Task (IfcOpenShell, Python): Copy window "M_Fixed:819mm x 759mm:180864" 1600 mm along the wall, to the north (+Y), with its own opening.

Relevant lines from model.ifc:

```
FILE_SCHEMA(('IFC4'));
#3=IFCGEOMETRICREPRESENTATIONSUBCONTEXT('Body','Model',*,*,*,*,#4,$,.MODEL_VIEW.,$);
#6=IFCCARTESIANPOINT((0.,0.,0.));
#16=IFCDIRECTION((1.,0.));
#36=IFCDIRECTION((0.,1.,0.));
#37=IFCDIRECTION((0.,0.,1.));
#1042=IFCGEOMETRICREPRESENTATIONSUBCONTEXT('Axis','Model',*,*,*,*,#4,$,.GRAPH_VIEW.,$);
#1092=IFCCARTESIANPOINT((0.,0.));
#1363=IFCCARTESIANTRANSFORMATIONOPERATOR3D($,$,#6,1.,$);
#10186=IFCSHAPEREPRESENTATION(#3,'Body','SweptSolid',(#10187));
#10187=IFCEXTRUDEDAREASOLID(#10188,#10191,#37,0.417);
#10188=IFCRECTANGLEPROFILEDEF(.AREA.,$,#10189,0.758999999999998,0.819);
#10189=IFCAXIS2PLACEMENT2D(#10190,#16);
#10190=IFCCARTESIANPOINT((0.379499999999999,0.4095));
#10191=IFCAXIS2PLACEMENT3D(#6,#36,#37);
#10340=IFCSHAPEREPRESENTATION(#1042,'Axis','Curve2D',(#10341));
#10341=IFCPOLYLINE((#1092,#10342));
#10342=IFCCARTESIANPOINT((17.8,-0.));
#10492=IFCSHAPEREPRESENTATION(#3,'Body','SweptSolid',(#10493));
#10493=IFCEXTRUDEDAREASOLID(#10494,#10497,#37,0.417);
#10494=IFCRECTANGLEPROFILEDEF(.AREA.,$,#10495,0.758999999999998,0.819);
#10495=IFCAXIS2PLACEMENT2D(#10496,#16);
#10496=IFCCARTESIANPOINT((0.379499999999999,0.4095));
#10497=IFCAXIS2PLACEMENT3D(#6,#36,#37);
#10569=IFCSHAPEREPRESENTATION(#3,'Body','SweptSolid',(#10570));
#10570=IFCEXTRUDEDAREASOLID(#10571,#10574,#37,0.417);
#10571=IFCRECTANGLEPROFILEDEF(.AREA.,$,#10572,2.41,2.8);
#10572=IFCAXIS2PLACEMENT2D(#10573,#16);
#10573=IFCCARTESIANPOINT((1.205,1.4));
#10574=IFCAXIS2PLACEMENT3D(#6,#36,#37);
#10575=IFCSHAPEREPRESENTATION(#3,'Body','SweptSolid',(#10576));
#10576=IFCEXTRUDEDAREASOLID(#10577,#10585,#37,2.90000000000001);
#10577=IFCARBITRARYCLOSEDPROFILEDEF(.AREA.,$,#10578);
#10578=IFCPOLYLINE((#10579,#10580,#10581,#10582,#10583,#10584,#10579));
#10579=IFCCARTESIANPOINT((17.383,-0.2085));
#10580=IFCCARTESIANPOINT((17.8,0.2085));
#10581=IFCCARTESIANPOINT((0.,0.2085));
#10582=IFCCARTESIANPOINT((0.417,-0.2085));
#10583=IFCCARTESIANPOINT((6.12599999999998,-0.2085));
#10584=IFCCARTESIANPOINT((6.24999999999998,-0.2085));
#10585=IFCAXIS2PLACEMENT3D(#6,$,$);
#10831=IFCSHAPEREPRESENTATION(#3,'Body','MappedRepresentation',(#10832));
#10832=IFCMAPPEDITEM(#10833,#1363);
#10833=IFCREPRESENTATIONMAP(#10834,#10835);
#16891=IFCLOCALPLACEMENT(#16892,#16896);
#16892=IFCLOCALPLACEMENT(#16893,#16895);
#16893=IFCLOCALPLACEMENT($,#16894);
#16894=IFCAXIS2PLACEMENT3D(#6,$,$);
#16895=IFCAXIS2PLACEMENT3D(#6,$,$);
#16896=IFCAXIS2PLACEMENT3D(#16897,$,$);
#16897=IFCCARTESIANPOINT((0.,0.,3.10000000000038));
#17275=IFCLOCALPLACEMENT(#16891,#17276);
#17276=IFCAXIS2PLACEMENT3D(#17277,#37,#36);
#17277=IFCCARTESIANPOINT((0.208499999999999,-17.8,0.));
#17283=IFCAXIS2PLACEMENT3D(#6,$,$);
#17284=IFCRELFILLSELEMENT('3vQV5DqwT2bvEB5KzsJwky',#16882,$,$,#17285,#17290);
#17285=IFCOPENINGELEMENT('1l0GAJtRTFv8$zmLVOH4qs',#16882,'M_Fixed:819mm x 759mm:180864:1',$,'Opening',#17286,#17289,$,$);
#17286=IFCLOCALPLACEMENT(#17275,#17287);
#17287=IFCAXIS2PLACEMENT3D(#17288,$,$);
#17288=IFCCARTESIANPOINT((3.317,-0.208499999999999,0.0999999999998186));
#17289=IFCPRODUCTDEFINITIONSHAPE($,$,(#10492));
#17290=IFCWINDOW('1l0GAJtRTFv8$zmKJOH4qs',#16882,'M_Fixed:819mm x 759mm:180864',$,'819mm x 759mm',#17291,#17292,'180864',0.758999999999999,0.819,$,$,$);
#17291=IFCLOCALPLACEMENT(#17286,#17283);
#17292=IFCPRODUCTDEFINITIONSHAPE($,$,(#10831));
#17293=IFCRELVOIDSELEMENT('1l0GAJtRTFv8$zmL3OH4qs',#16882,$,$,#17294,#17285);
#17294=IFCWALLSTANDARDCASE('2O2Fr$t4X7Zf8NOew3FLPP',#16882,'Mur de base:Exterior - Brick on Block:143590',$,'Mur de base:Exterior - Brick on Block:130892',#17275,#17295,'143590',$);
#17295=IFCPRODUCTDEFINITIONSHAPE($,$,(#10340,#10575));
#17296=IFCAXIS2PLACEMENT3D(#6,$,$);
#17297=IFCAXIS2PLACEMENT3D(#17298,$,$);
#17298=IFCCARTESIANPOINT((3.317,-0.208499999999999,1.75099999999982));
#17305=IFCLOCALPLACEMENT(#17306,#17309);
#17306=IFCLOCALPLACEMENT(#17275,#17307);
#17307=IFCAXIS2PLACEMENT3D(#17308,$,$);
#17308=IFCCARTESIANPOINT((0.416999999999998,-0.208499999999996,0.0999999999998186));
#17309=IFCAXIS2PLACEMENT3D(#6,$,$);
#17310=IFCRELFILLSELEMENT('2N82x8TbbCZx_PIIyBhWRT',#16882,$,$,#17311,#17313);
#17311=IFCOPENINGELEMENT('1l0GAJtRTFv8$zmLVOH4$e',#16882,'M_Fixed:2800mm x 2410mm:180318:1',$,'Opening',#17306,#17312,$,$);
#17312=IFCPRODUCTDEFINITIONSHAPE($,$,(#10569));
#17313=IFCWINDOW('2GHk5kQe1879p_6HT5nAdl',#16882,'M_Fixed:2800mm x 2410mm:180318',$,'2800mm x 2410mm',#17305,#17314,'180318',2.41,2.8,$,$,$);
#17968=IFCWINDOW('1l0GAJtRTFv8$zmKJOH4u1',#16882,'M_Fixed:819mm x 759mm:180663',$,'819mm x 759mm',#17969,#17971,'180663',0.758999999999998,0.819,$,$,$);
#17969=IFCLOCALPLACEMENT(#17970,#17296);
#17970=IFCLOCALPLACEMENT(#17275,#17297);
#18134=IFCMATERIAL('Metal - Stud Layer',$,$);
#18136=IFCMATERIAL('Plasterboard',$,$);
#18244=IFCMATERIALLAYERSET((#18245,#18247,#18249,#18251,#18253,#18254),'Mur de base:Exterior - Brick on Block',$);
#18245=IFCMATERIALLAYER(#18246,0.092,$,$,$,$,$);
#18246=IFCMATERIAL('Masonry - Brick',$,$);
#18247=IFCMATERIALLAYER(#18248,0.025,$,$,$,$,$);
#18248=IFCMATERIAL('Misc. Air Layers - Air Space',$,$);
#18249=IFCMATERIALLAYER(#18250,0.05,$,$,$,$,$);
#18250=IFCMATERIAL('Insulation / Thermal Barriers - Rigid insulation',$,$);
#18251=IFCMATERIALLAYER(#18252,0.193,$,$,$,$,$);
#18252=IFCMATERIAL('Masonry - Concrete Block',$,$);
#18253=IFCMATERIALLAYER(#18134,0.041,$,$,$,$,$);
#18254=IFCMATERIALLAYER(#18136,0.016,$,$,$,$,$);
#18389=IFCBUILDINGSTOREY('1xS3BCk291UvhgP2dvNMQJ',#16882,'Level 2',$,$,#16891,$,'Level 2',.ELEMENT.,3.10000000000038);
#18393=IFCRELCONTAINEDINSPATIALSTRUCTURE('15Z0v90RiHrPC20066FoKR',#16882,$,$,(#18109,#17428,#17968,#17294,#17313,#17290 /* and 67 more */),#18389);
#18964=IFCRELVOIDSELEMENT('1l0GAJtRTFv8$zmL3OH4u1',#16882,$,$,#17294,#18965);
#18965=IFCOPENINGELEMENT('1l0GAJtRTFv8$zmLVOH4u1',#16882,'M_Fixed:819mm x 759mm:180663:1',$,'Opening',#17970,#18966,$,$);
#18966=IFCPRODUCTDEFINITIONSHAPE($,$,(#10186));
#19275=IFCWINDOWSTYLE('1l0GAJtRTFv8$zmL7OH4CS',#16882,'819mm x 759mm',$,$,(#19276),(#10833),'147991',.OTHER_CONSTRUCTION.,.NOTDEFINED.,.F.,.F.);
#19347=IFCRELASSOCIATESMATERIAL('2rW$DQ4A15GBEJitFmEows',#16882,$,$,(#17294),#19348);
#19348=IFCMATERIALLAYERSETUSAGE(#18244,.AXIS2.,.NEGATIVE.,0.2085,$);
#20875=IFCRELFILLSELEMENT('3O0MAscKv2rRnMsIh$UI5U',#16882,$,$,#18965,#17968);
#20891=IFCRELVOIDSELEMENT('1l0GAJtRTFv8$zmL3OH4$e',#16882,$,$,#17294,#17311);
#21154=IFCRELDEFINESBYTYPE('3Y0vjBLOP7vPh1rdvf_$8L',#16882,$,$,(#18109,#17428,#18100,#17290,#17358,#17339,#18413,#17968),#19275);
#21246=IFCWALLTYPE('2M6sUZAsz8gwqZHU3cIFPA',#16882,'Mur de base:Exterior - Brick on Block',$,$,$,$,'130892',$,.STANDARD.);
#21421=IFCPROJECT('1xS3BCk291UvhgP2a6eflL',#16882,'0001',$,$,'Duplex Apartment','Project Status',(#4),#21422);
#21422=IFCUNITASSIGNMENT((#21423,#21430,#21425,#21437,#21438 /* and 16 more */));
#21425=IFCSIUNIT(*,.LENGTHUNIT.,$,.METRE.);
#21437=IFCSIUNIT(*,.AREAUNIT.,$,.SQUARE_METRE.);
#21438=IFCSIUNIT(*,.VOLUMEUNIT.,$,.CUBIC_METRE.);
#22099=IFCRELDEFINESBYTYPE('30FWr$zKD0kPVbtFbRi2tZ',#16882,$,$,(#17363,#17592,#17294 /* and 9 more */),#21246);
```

```python
import ifcopenshell
import ifcopenshell.api.feature
import ifcopenshell.api.geometry
import ifcopenshell.api.root
import ifcopenshell.geom
import ifcopenshell.util.element
import ifcopenshell.util.placement
import ifcopenshell.util.shape
import ifcopenshell.util.unit

model = ifcopenshell.open("model.ifc")
unit_scale = ifcopenshell.util.unit.calculate_unit_scale(model)
settings = ifcopenshell.geom.settings()


def volume(element):
    """Net volume in cubic metres, openings subtracted."""
    shape = ifcopenshell.geom.create_shape(settings, element)
    return ifcopenshell.util.shape.get_volume(shape.geometry)


def reuse_history(source, copy):
    """copy_class also copies each property set's owner history, people and application; keep the originals."""
    for rel in copy.IsDefinedBy:
        if rel.is_a("IfcRelDefinesByProperties") and (history := rel.RelatingPropertyDefinition.OwnerHistory):
            rel.RelatingPropertyDefinition.OwnerHistory = source.OwnerHistory
            ifcopenshell.util.element.remove_deep2(model, history)


window = model.by_id(17290)
opening = window.FillsVoids[0].RelatingOpeningElement
wall = opening.VoidsElements[0].RelatingBuildingElement
before = volume(wall)
shift = ifcopenshell.util.placement.get_local_placement(wall.ObjectPlacement)[:3, 0] * 1.6 / unit_scale

# copy_class copies the void relationship, type, container and properties, but no geometry.
new_opening = ifcopenshell.api.root.copy_class(model, product=opening)
new_opening.Representation = ifcopenshell.util.element.copy_deep(
    model, opening.Representation, exclude=["IfcGeometricRepresentationContext", "IfcRepresentationMap"]
)
new_opening.Name = "M_Fixed:819mm x 759mm"
new_window = ifcopenshell.api.root.copy_class(model, product=window)
new_window.Representation = ifcopenshell.util.element.copy_deep(
    model, window.Representation, exclude=["IfcGeometricRepresentationContext", "IfcRepresentationMap"]
)
new_window.Name = "M_Fixed:819mm x 759mm"
new_window.Tag = None
reuse_history(window, new_window)
ifcopenshell.api.feature.add_filling(model, opening=new_opening, element=new_window)

for old, new in ((opening, new_opening), (window, new_window)):
    matrix = ifcopenshell.util.placement.get_local_placement(old.ObjectPlacement)
    matrix[:3, 3] += shift
    ifcopenshell.api.geometry.edit_object_placement(model, product=new, matrix=matrix, is_si=False)

after = volume(wall)

print(f"wall volume {before:.3f} -> {after:.3f} m3")

model.write("model_edited.ifc")
```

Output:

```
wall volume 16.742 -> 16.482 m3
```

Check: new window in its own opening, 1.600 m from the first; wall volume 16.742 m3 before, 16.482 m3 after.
